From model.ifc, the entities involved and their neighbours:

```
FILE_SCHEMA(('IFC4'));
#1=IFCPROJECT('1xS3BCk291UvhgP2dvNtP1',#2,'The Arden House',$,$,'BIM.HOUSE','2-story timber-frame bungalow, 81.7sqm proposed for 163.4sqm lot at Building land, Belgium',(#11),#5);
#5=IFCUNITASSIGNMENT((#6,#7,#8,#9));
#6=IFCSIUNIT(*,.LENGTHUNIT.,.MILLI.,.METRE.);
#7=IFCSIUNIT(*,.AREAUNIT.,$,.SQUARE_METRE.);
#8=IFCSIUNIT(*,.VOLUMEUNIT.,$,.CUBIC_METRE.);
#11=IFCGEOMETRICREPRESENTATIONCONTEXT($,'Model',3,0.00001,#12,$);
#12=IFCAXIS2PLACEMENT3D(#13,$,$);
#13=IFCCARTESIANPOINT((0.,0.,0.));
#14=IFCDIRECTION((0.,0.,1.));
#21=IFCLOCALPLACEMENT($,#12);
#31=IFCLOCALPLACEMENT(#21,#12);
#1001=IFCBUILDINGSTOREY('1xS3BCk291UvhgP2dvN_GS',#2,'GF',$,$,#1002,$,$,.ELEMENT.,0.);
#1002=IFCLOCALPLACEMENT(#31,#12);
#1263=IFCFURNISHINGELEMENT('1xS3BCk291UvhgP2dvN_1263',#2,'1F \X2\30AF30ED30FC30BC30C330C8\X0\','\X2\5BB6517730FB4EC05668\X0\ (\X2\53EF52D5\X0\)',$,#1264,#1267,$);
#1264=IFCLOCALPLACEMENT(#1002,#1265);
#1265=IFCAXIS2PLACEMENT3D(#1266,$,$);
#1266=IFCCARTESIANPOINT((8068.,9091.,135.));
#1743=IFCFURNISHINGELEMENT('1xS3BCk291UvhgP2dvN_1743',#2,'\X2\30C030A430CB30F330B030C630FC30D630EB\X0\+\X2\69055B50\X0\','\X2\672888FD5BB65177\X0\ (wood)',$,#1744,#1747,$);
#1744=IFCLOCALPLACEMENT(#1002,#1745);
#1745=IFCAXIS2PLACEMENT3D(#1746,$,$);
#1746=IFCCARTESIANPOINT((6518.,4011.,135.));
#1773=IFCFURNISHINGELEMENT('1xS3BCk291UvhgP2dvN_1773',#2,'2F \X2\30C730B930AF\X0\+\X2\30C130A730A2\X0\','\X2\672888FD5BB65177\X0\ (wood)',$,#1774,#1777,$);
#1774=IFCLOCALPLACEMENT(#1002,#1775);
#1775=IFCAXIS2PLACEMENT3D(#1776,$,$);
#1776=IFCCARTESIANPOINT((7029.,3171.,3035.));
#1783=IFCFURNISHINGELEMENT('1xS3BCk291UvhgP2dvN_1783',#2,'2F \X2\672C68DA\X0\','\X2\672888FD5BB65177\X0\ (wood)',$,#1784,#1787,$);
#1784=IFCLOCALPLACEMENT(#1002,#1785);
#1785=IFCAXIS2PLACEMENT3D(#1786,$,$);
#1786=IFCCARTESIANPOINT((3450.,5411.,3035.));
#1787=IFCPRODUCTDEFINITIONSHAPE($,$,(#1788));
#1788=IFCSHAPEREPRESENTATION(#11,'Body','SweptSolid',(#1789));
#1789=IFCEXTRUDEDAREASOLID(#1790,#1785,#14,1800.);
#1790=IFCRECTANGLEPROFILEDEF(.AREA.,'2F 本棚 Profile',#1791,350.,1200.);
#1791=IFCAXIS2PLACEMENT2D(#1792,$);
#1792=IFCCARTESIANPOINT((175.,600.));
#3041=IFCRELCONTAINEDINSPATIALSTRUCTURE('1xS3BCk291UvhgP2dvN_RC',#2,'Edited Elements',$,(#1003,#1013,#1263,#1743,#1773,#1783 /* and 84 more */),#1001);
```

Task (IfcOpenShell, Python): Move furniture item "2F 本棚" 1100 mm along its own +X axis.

```python
import ifcopenshell
import ifcopenshell.api.geometry
import ifcopenshell.util.placement
import ifcopenshell.util.unit

model = ifcopenshell.open("model.ifc")
unit_scale = ifcopenshell.util.unit.calculate_unit_scale(model)

item = model.by_guid("1xS3BCk291UvhgP2dvN_1783")
matrix = ifcopenshell.util.placement.get_local_placement(item.ObjectPlacement)
matrix[:3, 3] += matrix[:3, 0] * 1.1 / unit_scale
ifcopenshell.api.geometry.edit_object_placement(model, product=item, matrix=matrix, is_si=False)

print(ifcopenshell.util.placement.get_local_placement(item.ObjectPlacement).round(3) + 0.0)

model.write("model-out.ifc")
```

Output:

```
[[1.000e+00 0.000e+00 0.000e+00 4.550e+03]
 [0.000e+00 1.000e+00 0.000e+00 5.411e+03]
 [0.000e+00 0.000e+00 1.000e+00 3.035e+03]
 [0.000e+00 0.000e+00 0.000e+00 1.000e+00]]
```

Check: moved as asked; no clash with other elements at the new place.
